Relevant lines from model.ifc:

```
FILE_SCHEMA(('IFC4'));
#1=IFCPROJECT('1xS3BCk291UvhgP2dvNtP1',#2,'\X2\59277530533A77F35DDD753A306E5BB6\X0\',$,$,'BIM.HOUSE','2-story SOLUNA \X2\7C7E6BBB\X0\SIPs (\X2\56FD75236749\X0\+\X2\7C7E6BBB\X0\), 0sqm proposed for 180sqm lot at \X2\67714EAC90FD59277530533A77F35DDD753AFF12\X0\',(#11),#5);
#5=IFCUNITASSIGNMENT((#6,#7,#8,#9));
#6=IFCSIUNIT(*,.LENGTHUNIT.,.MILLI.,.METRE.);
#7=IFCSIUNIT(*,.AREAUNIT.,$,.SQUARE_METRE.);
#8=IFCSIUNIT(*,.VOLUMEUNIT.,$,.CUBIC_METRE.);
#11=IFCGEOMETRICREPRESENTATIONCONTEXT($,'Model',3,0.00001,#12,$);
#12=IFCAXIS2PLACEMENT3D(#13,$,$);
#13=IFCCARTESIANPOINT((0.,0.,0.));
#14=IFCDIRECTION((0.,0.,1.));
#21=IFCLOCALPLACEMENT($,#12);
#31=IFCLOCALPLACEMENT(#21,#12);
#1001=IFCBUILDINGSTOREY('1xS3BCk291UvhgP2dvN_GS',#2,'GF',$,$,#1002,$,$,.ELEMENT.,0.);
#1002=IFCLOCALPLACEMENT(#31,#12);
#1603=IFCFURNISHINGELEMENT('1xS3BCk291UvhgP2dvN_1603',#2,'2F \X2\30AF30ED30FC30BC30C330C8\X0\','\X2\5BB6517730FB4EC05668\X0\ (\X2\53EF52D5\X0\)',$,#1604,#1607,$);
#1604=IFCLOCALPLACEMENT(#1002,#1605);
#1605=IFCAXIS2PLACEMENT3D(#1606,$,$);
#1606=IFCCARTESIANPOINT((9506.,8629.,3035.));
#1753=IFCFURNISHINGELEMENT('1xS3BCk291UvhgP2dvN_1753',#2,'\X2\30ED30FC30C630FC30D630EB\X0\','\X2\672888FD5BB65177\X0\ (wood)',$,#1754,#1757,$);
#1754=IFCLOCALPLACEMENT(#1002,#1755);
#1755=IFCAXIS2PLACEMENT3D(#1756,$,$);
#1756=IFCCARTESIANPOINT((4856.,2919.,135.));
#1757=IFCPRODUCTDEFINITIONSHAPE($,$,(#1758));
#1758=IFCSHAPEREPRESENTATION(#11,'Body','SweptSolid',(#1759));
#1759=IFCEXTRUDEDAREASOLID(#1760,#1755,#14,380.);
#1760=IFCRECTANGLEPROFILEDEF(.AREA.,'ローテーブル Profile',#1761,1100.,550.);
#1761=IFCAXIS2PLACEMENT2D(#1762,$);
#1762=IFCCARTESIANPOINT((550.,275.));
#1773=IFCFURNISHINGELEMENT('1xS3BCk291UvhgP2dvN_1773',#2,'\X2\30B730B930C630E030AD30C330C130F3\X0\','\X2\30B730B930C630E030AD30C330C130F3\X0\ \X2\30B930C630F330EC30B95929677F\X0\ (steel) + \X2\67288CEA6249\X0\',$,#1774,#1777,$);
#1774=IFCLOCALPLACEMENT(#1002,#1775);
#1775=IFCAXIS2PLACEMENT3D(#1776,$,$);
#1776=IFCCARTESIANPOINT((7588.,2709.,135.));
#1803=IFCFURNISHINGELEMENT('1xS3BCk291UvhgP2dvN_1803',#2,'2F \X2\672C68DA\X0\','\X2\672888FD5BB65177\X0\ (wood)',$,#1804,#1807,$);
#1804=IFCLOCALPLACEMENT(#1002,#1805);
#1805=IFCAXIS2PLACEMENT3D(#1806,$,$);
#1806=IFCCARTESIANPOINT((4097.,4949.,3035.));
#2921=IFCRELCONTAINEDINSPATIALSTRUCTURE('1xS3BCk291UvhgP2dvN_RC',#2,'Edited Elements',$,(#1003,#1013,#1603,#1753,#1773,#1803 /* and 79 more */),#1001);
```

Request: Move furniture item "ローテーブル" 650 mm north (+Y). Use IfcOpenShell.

```python
import ifcopenshell
import ifcopenshell.api.geometry
import ifcopenshell.util.placement

model = ifcopenshell.open("model.ifc")

item = model.by_guid("1xS3BCk291UvhgP2dvN_1753")
matrix = ifcopenshell.util.placement.get_local_placement(item.ObjectPlacement)
matrix[1, 3] += 650.0
ifcopenshell.api.geometry.edit_object_placement(model, product=item, matrix=matrix, is_si=False)

print(ifcopenshell.util.placement.get_local_placement(item.ObjectPlacement).round(3) + 0.0)

model.write("model_rev.ifc")
```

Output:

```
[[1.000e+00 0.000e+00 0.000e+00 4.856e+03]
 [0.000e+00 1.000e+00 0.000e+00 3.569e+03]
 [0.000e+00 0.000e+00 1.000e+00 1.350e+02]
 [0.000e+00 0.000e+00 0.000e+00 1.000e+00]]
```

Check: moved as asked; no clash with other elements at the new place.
